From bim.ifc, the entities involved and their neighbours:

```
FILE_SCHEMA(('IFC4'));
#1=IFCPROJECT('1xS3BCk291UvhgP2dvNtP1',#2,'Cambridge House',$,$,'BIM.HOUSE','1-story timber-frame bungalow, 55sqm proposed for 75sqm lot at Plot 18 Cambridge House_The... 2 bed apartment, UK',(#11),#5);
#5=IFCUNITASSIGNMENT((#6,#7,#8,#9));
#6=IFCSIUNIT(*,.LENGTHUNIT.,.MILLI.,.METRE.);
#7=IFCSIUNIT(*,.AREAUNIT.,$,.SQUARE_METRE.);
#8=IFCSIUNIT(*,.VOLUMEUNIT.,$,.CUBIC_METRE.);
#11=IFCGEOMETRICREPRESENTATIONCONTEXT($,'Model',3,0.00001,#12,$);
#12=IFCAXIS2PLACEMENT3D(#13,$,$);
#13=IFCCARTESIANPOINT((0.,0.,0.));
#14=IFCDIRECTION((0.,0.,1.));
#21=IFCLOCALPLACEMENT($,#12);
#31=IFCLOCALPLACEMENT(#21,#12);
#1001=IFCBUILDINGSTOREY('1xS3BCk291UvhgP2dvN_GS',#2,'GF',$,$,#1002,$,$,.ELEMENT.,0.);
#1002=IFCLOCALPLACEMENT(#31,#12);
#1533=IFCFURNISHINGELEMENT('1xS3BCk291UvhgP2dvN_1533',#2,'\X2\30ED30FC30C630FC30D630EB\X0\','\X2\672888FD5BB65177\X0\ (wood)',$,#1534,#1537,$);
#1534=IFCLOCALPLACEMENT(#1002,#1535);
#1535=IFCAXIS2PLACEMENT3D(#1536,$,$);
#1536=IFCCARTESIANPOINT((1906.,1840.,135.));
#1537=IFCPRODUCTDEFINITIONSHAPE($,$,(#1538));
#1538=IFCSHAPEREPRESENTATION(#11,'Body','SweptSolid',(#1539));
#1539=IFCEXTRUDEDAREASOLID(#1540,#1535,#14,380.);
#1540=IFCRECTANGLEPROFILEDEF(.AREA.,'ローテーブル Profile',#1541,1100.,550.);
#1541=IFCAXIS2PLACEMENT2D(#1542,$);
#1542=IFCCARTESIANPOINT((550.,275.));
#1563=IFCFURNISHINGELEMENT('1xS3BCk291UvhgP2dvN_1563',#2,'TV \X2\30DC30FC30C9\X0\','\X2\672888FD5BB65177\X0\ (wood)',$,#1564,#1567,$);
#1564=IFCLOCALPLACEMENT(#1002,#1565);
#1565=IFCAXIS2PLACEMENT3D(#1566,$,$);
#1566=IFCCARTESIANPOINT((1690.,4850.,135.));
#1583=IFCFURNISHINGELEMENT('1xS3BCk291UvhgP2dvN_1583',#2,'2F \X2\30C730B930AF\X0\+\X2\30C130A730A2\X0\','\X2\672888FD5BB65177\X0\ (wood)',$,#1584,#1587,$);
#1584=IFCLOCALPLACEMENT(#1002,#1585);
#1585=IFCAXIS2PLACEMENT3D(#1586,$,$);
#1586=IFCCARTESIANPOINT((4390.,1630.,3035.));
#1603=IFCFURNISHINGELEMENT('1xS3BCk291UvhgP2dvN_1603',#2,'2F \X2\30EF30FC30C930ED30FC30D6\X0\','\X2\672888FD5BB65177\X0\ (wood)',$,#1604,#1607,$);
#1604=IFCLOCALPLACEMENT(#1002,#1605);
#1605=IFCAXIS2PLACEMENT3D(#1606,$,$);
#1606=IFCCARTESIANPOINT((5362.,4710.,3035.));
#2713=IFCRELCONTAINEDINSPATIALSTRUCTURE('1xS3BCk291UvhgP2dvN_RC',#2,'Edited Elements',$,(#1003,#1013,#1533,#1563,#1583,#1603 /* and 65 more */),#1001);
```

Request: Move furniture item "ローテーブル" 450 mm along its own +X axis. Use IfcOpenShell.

```python
import ifcopenshell
import ifcopenshell.api.geometry
import ifcopenshell.util.placement

model = ifcopenshell.open("bim.ifc")

item = model.by_guid("1xS3BCk291UvhgP2dvN_1533")
matrix = ifcopenshell.util.placement.get_local_placement(item.ObjectPlacement)
matrix[:3, 3] += matrix[:3, 0] * 450.0
ifcopenshell.api.geometry.edit_object_placement(model, product=item, matrix=matrix, is_si=False)

print(ifcopenshell.util.placement.get_local_placement(item.ObjectPlacement).round(3) + 0.0)

model.write("bim-out.ifc")
```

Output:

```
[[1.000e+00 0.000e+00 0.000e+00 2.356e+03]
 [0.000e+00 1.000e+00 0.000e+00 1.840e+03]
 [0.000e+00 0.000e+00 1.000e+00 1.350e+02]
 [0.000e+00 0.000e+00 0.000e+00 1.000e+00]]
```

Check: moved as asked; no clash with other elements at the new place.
